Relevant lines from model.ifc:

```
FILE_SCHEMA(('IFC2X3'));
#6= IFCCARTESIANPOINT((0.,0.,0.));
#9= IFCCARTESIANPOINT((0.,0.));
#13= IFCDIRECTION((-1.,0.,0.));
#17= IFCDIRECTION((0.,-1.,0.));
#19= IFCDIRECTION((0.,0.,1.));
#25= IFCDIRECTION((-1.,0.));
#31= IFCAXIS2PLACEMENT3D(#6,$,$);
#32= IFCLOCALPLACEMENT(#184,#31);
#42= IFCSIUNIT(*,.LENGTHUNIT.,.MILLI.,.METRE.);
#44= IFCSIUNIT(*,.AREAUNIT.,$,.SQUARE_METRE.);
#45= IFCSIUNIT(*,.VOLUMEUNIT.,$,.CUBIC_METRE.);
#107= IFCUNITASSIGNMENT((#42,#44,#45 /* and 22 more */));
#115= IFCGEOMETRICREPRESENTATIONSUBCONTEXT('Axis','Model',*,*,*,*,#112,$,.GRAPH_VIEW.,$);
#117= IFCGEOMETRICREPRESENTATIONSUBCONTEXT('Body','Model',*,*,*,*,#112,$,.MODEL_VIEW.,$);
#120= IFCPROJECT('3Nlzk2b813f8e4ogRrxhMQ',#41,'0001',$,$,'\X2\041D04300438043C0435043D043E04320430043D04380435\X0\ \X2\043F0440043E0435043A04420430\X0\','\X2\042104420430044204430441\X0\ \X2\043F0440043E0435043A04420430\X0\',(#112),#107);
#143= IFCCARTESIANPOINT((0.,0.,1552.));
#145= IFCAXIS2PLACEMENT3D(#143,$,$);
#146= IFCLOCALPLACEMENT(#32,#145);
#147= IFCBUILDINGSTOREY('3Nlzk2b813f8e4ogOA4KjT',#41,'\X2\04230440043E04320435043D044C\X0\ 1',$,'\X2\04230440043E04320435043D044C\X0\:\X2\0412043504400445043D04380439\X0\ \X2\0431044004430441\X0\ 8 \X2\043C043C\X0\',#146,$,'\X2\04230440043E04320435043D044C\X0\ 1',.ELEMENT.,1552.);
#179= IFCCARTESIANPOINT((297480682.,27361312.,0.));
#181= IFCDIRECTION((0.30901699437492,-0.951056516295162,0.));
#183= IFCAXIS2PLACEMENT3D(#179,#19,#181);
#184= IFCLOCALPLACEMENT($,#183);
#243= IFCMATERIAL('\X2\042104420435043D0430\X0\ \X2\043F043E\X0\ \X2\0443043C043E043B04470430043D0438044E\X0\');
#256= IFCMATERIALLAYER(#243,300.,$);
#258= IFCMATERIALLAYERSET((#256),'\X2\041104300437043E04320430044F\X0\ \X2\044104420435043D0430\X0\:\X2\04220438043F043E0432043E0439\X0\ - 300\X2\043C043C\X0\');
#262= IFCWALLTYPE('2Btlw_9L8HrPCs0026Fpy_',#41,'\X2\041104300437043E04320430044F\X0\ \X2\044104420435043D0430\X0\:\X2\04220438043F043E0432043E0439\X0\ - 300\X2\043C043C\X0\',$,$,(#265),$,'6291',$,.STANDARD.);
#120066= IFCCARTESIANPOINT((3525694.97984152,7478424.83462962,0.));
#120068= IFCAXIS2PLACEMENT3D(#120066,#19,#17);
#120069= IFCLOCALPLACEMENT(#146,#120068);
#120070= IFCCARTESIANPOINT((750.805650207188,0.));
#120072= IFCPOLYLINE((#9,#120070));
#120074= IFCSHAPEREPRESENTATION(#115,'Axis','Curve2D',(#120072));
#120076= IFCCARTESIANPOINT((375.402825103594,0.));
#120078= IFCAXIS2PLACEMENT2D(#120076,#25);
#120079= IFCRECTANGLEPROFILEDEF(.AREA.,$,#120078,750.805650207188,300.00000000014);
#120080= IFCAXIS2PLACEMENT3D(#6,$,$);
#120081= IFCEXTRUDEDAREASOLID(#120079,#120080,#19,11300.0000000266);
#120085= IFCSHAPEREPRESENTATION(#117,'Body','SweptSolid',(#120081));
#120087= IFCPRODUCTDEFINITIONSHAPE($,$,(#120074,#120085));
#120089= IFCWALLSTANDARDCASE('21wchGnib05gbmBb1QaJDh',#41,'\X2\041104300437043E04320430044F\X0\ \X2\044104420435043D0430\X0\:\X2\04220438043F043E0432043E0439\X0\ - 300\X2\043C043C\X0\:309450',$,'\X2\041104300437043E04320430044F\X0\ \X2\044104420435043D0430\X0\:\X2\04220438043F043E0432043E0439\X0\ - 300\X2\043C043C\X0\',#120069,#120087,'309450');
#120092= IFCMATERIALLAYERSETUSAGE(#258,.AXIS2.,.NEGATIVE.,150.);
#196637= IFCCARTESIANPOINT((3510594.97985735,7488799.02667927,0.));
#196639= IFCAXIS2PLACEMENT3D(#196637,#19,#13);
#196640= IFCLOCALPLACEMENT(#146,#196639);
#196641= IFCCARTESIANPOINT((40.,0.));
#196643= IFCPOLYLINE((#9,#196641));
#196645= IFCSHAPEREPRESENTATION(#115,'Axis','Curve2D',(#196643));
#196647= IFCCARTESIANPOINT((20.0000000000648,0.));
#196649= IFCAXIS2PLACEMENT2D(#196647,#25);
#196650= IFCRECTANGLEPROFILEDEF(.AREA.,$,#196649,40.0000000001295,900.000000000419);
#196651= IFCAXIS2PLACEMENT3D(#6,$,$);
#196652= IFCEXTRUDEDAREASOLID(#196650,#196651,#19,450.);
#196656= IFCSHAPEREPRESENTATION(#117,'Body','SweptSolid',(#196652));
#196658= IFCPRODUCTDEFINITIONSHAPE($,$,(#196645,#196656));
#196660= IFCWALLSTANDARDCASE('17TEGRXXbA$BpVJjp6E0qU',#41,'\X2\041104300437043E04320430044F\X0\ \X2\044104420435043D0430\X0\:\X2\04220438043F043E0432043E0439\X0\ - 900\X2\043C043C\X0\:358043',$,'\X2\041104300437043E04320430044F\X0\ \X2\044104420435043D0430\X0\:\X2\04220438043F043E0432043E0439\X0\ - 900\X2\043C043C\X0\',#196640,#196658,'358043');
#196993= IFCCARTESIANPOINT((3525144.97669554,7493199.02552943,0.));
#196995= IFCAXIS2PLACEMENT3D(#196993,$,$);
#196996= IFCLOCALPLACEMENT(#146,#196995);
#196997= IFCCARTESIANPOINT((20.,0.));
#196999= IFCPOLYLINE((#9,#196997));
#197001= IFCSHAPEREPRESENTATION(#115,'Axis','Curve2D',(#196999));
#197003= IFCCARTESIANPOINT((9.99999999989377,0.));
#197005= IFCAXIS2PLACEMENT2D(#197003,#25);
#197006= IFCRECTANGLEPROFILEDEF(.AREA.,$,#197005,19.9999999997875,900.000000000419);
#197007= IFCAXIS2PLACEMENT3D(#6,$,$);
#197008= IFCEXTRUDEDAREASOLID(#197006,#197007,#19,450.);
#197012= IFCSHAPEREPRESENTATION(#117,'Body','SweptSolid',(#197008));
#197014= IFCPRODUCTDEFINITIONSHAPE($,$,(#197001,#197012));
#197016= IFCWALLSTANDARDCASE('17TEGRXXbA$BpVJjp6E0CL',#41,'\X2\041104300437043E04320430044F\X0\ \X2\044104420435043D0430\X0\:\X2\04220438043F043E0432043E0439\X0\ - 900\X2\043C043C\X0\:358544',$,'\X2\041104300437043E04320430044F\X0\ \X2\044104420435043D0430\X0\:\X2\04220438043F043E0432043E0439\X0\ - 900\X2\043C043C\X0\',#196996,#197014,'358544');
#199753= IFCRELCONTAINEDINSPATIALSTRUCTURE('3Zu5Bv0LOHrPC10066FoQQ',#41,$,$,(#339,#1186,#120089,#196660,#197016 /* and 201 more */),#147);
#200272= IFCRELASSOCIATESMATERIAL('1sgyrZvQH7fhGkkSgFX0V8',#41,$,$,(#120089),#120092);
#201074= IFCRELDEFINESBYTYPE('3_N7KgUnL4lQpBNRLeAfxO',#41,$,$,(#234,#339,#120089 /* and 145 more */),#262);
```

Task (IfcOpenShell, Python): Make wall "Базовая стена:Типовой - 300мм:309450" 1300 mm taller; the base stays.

```python
import ifcopenshell
import ifcopenshell.geom
import ifcopenshell.util.representation
import ifcopenshell.util.shape

model = ifcopenshell.open("model.ifc")
settings = ifcopenshell.geom.settings()


def volume(element):
    """Net volume in cubic metres, openings subtracted."""
    shape = ifcopenshell.geom.create_shape(settings, element)
    return ifcopenshell.util.shape.get_volume(shape.geometry)


wall = model.by_guid("21wchGnib05gbmBb1QaJDh")
before = volume(wall)

body = ifcopenshell.util.representation.get_representation(wall, "Model", "Body")
solid = body.Items[0]
old_height = solid.Depth
solid.Depth += 1300.0
after = volume(wall)

print(f"height {old_height:g} -> {solid.Depth:g}, volume {before:.3f} -> {after:.3f} m3")

model.write("model_updated.ifc")
```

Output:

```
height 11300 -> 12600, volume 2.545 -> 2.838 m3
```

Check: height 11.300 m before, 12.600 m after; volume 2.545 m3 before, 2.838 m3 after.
